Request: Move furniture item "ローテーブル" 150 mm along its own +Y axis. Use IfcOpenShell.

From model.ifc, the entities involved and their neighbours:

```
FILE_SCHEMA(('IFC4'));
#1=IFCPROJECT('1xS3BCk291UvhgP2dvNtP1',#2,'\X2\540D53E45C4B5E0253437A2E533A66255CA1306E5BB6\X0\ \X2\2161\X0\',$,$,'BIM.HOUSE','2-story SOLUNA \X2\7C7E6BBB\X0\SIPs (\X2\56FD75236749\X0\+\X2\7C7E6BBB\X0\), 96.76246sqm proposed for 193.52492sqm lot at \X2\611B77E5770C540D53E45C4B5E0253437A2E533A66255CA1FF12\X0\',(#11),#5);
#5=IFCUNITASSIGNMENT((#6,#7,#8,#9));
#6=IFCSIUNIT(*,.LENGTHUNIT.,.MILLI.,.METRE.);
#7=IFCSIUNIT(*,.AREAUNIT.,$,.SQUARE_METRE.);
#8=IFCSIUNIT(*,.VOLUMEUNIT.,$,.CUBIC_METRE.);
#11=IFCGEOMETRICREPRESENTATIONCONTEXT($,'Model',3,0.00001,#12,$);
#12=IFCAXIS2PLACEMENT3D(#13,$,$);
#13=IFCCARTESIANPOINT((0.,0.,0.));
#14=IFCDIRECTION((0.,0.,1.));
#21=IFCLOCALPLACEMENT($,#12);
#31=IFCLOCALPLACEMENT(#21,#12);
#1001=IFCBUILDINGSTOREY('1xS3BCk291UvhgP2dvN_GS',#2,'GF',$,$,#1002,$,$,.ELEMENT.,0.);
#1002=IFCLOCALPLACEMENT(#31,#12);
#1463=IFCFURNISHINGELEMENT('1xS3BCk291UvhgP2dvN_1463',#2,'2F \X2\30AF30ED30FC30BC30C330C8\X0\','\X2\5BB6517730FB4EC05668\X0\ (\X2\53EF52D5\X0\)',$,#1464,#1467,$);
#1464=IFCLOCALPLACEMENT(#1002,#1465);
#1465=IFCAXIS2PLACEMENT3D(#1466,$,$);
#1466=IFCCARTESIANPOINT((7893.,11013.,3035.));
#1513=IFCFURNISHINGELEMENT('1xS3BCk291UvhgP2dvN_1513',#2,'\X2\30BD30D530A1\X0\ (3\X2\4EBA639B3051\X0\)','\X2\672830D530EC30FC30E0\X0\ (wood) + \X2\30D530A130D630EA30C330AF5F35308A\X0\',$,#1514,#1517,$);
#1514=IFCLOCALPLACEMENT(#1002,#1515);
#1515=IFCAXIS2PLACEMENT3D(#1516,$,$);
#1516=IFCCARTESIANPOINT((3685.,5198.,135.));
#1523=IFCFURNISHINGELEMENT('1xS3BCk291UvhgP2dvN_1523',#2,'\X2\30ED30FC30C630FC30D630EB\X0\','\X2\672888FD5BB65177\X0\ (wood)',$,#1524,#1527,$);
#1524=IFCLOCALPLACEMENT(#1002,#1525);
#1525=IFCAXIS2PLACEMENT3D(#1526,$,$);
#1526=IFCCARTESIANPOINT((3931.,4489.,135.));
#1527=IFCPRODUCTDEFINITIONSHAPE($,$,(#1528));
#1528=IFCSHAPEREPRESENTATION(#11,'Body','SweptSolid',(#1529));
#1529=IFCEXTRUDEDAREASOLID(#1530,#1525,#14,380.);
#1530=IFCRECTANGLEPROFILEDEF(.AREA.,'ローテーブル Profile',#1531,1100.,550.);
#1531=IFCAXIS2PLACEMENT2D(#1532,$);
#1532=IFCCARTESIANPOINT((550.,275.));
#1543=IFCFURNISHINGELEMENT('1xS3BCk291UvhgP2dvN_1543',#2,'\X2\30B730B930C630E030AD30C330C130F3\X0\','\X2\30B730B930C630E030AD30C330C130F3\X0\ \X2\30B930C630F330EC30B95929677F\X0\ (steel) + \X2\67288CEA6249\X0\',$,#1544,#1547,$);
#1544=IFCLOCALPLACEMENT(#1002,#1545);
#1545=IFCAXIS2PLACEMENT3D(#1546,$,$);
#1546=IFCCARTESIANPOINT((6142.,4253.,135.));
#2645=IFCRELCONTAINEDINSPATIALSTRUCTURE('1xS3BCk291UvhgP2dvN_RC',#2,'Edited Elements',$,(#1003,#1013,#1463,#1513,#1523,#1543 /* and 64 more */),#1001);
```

```python
import ifcopenshell
import ifcopenshell.api.geometry
import ifcopenshell.util.placement

model = ifcopenshell.open("model.ifc")

item = model.by_guid("1xS3BCk291UvhgP2dvN_1523")
matrix = ifcopenshell.util.placement.get_local_placement(item.ObjectPlacement)
matrix[:3, 3] += matrix[:3, 1] * 150.0
ifcopenshell.api.geometry.edit_object_placement(model, product=item, matrix=matrix, is_si=False)

print(ifcopenshell.util.placement.get_local_placement(item.ObjectPlacement).round(3) + 0.0)

model.write("model_v2.ifc")
```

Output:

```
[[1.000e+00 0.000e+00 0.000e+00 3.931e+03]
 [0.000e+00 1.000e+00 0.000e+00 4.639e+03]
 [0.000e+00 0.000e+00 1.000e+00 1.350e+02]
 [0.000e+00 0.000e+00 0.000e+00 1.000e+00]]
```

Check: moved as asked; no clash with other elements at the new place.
